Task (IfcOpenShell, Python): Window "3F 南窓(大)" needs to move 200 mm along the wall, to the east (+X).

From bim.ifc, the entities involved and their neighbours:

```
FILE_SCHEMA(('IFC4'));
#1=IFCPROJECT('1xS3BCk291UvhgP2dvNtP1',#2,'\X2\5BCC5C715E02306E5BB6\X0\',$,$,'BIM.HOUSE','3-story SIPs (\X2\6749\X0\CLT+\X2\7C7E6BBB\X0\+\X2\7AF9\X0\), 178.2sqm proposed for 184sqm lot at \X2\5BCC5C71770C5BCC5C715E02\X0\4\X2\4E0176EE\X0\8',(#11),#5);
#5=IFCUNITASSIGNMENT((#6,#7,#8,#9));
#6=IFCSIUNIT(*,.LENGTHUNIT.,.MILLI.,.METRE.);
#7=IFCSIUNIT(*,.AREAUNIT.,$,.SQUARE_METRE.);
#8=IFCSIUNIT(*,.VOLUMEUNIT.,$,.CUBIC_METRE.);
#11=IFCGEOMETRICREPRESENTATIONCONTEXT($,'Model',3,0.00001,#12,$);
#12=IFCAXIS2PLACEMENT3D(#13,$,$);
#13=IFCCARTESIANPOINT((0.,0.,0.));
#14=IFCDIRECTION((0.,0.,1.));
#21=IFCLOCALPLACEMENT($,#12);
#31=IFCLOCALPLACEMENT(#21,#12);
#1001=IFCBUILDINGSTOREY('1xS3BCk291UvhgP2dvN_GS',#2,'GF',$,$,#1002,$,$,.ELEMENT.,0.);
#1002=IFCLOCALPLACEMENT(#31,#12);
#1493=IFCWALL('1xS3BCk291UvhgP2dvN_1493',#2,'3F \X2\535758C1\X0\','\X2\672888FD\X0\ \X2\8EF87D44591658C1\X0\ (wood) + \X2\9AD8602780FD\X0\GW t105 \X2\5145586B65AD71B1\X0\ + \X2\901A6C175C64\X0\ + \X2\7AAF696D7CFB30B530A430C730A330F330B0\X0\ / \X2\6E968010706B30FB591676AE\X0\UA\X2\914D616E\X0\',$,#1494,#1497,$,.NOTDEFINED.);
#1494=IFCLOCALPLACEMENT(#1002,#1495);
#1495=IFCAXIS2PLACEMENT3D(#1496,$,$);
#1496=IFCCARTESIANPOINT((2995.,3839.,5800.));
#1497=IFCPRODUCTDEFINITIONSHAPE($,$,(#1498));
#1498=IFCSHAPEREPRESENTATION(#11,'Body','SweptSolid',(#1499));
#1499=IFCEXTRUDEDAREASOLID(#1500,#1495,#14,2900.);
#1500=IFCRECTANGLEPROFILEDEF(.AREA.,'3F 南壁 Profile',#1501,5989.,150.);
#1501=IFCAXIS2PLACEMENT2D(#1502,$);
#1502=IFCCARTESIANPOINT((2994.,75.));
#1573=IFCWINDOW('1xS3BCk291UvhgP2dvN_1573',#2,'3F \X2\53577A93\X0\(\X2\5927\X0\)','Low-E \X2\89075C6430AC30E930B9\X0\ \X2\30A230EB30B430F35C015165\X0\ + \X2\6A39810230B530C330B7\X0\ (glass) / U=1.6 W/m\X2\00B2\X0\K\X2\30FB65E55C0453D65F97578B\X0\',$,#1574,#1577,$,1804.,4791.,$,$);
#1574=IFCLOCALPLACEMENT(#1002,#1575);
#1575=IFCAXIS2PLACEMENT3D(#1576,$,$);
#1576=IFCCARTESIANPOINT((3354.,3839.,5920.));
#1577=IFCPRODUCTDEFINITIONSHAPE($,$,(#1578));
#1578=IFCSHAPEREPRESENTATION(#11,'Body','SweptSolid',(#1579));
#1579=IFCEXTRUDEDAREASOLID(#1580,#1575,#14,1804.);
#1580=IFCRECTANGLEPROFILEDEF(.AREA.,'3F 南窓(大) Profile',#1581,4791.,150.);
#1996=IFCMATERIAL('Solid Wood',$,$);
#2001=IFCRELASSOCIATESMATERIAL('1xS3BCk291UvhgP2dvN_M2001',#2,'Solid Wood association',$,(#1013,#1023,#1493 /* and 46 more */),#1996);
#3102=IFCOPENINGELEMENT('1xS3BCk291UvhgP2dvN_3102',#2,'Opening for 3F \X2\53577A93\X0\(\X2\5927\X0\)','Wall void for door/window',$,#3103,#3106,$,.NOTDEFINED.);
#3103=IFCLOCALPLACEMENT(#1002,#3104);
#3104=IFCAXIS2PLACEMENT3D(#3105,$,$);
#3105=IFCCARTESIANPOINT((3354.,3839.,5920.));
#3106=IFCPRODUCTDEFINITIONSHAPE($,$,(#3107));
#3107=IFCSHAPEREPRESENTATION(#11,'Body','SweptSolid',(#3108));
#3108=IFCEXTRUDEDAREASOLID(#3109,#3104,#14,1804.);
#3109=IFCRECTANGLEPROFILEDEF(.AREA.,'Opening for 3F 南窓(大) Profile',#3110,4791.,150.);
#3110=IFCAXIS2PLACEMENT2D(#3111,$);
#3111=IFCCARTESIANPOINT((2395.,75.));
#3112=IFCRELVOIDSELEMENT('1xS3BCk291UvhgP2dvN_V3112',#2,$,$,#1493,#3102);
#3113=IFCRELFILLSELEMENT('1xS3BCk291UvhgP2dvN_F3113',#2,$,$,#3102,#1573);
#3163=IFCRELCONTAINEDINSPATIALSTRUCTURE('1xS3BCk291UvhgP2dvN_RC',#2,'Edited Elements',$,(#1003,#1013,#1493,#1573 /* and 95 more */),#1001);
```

```python
import ifcopenshell
import ifcopenshell.api.geometry
import ifcopenshell.util.placement
import ifcopenshell.util.unit

model = ifcopenshell.open("bim.ifc")
unit_scale = ifcopenshell.util.unit.calculate_unit_scale(model)

window = model.by_guid("1xS3BCk291UvhgP2dvN_1573")
opening = window.FillsVoids[0].RelatingOpeningElement
wall = opening.VoidsElements[0].RelatingBuildingElement

wall_matrix = ifcopenshell.util.placement.get_local_placement(wall.ObjectPlacement)
shift = wall_matrix[:3, 0] * 0.2 / unit_scale
before = ifcopenshell.util.placement.get_local_placement(window.ObjectPlacement)[:3, 3].copy()

# The window is not placed relative to its opening, so move both.
for product in (opening, window):
    matrix = ifcopenshell.util.placement.get_local_placement(product.ObjectPlacement)
    matrix[:3, 3] += shift
    ifcopenshell.api.geometry.edit_object_placement(model, product=product, matrix=matrix, is_si=False)

after = ifcopenshell.util.placement.get_local_placement(window.ObjectPlacement)[:3, 3]
print("window moved by", (after - before).round(3) + 0.0)

model.write("bim_updated.ifc")
```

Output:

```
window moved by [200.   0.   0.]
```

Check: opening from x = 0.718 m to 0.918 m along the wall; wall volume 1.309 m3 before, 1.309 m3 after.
